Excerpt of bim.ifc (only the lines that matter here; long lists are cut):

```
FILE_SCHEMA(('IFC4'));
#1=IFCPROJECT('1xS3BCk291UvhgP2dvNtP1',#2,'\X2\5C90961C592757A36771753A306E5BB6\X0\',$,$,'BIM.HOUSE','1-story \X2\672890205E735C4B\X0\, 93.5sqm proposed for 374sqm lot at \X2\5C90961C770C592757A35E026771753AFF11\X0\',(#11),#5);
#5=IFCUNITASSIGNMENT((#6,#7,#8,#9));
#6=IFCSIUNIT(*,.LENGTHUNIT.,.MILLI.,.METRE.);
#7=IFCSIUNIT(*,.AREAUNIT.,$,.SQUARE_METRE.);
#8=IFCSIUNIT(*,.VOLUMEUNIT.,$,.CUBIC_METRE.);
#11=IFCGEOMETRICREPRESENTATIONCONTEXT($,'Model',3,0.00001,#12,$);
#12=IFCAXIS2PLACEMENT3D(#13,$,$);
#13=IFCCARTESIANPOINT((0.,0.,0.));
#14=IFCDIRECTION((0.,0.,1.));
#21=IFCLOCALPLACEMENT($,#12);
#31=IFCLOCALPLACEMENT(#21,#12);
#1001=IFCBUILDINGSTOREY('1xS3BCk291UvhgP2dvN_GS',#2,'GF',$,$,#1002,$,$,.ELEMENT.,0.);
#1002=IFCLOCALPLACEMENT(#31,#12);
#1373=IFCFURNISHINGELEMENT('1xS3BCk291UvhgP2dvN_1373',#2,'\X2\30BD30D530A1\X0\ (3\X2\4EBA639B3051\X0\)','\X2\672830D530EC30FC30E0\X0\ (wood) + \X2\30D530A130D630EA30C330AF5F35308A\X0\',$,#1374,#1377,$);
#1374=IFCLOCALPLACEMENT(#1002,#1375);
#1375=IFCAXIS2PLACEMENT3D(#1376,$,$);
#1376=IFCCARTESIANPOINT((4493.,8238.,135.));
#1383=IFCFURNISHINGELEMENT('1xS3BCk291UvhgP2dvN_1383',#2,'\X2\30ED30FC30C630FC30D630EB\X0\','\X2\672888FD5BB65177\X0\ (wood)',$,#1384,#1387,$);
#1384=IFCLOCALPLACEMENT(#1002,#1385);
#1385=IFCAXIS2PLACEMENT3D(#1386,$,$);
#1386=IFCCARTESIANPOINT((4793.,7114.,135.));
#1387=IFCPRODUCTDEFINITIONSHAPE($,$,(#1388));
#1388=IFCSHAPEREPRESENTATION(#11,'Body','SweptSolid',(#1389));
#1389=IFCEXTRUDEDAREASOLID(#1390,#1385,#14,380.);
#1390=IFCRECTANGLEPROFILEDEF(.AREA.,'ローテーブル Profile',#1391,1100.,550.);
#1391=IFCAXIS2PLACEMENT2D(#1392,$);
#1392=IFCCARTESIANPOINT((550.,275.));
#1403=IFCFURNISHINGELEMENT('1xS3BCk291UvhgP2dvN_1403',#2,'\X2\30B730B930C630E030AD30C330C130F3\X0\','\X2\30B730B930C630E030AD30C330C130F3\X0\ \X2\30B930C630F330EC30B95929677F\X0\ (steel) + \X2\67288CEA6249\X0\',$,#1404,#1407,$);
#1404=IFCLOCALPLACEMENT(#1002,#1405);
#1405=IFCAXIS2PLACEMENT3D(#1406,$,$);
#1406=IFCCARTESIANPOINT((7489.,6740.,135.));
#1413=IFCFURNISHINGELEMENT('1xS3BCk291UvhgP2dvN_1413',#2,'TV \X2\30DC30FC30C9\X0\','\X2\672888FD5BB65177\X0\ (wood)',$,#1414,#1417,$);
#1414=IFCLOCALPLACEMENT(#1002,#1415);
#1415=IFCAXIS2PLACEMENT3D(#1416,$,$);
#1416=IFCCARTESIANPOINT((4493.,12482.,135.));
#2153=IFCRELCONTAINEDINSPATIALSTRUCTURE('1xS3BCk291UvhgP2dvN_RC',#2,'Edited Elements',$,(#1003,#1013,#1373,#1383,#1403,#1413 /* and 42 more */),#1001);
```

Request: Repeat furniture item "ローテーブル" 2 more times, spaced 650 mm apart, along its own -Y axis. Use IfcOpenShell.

```python
import ifcopenshell
import ifcopenshell.api.geometry
import ifcopenshell.api.root
import ifcopenshell.util.element
import ifcopenshell.util.placement

model = ifcopenshell.open("bim.ifc")


def reuse_history(source, copy):
    """copy_class also copies each property set's owner history, people and application; keep the originals."""
    for rel in copy.IsDefinedBy:
        if rel.is_a("IfcRelDefinesByProperties") and (history := rel.RelatingPropertyDefinition.OwnerHistory):
            rel.RelatingPropertyDefinition.OwnerHistory = source.OwnerHistory
            ifcopenshell.util.element.remove_deep2(model, history)


source = model.by_guid("1xS3BCk291UvhgP2dvN_1383")
base = ifcopenshell.util.placement.get_local_placement(source.ObjectPlacement)
step = -base[:3, 1] * 650.0

for i in range(1, 3):
    copy = ifcopenshell.api.root.copy_class(model, product=source)
    copy.Representation = ifcopenshell.util.element.copy_deep(
        model, source.Representation, exclude=["IfcGeometricRepresentationContext", "IfcRepresentationMap"]
    )
    reuse_history(source, copy)
    matrix = base.copy()
    matrix[:3, 3] += i * step
    print("added at", matrix[:3, 3].round(3) + 0.0)
    ifcopenshell.api.geometry.edit_object_placement(model, product=copy, matrix=matrix, is_si=False)

model.write("bim_v2.ifc")
```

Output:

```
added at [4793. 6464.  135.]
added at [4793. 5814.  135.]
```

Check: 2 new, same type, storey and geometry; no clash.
